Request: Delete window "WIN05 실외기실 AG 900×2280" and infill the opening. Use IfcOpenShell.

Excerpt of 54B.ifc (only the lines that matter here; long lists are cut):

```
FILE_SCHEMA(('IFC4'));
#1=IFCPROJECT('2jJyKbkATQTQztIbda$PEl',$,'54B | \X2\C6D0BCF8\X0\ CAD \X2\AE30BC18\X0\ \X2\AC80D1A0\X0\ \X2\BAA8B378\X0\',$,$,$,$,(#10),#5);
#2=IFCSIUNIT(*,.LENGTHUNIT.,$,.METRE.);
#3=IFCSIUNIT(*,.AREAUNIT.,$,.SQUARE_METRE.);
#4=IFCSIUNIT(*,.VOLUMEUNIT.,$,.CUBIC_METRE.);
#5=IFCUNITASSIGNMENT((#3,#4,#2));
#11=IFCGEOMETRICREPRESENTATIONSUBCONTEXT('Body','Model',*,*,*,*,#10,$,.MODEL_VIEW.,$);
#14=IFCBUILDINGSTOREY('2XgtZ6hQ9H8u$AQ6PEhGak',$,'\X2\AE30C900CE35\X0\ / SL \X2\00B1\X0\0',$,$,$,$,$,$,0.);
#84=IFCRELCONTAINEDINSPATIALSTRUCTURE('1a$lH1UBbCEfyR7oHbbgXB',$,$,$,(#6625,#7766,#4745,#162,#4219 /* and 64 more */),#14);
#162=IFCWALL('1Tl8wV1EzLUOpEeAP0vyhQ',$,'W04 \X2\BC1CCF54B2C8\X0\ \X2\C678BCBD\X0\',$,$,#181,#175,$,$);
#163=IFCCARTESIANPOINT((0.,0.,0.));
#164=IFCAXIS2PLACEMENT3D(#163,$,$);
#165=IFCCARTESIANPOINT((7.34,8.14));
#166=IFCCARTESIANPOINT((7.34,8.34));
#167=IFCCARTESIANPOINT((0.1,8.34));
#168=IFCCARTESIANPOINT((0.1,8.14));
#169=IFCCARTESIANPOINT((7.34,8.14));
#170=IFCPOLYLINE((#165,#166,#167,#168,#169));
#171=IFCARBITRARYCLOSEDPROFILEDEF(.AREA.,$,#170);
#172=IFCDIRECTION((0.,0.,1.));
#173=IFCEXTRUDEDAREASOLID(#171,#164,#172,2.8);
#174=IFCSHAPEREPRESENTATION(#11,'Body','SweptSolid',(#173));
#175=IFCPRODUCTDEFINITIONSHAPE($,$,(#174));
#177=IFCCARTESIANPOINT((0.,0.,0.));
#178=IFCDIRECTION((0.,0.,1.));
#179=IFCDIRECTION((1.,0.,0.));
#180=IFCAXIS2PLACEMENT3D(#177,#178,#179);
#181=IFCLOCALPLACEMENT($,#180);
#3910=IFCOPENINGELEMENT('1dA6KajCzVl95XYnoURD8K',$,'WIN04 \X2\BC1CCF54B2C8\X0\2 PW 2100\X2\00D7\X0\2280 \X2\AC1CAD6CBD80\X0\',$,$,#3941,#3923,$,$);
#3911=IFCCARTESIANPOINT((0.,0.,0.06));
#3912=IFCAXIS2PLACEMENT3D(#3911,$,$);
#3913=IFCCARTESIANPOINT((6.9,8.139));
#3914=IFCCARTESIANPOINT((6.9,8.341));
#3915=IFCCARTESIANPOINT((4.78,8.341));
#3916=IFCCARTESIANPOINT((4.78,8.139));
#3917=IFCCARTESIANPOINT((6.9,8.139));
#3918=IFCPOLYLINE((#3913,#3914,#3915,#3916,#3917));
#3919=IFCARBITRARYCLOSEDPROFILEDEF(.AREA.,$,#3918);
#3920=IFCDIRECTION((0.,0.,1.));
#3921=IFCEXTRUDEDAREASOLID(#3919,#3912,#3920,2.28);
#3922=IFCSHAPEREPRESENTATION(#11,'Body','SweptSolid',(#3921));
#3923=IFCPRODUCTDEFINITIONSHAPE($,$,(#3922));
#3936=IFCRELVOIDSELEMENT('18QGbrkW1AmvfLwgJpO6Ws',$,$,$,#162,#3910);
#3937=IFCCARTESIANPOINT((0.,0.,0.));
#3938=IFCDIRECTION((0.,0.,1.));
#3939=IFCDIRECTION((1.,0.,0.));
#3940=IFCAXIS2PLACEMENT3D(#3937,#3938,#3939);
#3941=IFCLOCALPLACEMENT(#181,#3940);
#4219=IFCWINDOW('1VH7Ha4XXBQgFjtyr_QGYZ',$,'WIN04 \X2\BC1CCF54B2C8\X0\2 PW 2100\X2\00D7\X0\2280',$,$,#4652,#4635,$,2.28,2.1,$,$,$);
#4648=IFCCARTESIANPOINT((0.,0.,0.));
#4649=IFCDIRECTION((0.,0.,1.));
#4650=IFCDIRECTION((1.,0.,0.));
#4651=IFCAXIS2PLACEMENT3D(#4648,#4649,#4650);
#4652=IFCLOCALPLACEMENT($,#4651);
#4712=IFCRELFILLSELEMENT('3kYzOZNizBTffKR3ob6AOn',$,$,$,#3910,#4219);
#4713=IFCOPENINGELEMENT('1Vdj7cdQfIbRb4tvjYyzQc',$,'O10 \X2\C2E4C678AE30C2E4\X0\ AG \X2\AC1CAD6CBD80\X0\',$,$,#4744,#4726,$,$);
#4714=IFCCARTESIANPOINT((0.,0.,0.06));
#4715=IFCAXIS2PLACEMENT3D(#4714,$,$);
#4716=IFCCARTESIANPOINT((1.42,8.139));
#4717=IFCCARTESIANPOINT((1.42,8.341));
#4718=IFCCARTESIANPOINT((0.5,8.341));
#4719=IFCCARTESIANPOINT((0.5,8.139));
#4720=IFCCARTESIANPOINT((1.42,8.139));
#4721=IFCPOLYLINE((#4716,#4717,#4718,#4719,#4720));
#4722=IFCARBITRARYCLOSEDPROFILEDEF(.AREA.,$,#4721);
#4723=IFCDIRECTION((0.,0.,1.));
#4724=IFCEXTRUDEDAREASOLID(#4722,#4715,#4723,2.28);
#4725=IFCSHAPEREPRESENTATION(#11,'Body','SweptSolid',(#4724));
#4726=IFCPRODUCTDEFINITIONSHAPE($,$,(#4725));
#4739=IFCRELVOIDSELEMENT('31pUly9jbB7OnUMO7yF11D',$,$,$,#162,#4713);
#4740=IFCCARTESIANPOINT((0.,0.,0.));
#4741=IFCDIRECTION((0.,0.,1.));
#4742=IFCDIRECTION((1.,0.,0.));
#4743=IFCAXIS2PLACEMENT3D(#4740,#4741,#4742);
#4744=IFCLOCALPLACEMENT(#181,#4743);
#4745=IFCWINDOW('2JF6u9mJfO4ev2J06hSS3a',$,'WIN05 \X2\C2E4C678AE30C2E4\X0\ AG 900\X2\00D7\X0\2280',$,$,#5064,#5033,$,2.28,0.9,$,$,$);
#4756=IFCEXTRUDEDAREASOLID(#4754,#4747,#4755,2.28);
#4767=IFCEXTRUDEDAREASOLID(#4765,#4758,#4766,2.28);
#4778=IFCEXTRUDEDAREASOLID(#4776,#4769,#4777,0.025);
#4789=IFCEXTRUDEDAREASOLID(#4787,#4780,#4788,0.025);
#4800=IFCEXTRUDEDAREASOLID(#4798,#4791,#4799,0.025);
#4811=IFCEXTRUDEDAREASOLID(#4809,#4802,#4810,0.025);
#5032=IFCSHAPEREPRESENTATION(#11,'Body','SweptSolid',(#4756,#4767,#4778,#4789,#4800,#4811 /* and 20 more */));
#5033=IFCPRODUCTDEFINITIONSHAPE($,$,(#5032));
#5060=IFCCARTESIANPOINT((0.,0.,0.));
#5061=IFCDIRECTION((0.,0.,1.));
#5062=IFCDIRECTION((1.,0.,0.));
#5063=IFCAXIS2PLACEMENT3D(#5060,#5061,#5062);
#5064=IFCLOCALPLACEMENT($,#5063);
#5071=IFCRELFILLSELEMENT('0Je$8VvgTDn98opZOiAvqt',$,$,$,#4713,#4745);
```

```python
import ifcopenshell
import ifcopenshell.api.feature
import ifcopenshell.api.root
import ifcopenshell.geom
import ifcopenshell.util.shape

model = ifcopenshell.open("54B.ifc")
settings = ifcopenshell.geom.settings()


def volume(element):
    """Net volume in cubic metres, openings subtracted."""
    shape = ifcopenshell.geom.create_shape(settings, element)
    return ifcopenshell.util.shape.get_volume(shape.geometry)


window = model.by_guid("2JF6u9mJfO4ev2J06hSS3a")
opening = window.FillsVoids[0].RelatingOpeningElement
wall = opening.VoidsElements[0].RelatingBuildingElement
before = volume(wall)

ifcopenshell.api.root.remove_product(model, product=window)
ifcopenshell.api.feature.remove_feature(model, feature=opening)

after = volume(wall)

print(f"wall volume {before:.3f} -> {after:.3f} m3")

model.write("54B_edited.ifc")
```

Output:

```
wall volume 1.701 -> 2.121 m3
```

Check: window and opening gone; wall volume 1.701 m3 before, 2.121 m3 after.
